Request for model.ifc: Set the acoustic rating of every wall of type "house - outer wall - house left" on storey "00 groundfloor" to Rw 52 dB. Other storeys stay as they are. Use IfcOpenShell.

First a look at what the model holds.

```python
import ifcopenshell
import ifcopenshell.util.element

model = ifcopenshell.open("model.ifc")
print(model.schema)
storey = next(s for s in model.by_type("IfcBuildingStorey") if s.Name == "00 groundfloor")
walls = [e for e in ifcopenshell.util.element.get_decomposition(storey) if e.is_a("IfcWall")]
seen = {}
for e in walls:
    element_type = ifcopenshell.util.element.get_type(e)
    key = (element_type.Name if element_type != e and element_type else None, ifcopenshell.util.element.get_pset(e, "Pset_WallCommon", "AcousticRating"))
    seen[key] = seen.get(key, 0) + 1
for (name, value), count in sorted(seen.items(), key=str):
    print(count, "x", name, "|", value)
```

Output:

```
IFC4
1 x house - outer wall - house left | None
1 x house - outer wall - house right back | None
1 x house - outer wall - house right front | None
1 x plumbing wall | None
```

```python
import ifcopenshell
import ifcopenshell.api.pset
import ifcopenshell.util.element

model = ifcopenshell.open("model.ifc")

storey = next(s for s in model.by_type("IfcBuildingStorey") if s.Name == "00 groundfloor")
walls = [e for e in ifcopenshell.util.element.get_decomposition(storey) if e.is_a("IfcWall")]

count = 0
for e in walls:
    element_type = ifcopenshell.util.element.get_type(e)
    if element_type in (None, e) or element_type.Name != "house - outer wall - house left":
        continue
    # add_pset returns the element's existing set when there is one.
    pset = ifcopenshell.api.pset.add_pset(model, product=e, name="Pset_WallCommon")
    ifcopenshell.api.pset.edit_pset(model, pset=pset, properties={"AcousticRating": "Rw 52 dB"})
    count += 1

print(count, "walls updated")

model.write("model-out.ifc")
```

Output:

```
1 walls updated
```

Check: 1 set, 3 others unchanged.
